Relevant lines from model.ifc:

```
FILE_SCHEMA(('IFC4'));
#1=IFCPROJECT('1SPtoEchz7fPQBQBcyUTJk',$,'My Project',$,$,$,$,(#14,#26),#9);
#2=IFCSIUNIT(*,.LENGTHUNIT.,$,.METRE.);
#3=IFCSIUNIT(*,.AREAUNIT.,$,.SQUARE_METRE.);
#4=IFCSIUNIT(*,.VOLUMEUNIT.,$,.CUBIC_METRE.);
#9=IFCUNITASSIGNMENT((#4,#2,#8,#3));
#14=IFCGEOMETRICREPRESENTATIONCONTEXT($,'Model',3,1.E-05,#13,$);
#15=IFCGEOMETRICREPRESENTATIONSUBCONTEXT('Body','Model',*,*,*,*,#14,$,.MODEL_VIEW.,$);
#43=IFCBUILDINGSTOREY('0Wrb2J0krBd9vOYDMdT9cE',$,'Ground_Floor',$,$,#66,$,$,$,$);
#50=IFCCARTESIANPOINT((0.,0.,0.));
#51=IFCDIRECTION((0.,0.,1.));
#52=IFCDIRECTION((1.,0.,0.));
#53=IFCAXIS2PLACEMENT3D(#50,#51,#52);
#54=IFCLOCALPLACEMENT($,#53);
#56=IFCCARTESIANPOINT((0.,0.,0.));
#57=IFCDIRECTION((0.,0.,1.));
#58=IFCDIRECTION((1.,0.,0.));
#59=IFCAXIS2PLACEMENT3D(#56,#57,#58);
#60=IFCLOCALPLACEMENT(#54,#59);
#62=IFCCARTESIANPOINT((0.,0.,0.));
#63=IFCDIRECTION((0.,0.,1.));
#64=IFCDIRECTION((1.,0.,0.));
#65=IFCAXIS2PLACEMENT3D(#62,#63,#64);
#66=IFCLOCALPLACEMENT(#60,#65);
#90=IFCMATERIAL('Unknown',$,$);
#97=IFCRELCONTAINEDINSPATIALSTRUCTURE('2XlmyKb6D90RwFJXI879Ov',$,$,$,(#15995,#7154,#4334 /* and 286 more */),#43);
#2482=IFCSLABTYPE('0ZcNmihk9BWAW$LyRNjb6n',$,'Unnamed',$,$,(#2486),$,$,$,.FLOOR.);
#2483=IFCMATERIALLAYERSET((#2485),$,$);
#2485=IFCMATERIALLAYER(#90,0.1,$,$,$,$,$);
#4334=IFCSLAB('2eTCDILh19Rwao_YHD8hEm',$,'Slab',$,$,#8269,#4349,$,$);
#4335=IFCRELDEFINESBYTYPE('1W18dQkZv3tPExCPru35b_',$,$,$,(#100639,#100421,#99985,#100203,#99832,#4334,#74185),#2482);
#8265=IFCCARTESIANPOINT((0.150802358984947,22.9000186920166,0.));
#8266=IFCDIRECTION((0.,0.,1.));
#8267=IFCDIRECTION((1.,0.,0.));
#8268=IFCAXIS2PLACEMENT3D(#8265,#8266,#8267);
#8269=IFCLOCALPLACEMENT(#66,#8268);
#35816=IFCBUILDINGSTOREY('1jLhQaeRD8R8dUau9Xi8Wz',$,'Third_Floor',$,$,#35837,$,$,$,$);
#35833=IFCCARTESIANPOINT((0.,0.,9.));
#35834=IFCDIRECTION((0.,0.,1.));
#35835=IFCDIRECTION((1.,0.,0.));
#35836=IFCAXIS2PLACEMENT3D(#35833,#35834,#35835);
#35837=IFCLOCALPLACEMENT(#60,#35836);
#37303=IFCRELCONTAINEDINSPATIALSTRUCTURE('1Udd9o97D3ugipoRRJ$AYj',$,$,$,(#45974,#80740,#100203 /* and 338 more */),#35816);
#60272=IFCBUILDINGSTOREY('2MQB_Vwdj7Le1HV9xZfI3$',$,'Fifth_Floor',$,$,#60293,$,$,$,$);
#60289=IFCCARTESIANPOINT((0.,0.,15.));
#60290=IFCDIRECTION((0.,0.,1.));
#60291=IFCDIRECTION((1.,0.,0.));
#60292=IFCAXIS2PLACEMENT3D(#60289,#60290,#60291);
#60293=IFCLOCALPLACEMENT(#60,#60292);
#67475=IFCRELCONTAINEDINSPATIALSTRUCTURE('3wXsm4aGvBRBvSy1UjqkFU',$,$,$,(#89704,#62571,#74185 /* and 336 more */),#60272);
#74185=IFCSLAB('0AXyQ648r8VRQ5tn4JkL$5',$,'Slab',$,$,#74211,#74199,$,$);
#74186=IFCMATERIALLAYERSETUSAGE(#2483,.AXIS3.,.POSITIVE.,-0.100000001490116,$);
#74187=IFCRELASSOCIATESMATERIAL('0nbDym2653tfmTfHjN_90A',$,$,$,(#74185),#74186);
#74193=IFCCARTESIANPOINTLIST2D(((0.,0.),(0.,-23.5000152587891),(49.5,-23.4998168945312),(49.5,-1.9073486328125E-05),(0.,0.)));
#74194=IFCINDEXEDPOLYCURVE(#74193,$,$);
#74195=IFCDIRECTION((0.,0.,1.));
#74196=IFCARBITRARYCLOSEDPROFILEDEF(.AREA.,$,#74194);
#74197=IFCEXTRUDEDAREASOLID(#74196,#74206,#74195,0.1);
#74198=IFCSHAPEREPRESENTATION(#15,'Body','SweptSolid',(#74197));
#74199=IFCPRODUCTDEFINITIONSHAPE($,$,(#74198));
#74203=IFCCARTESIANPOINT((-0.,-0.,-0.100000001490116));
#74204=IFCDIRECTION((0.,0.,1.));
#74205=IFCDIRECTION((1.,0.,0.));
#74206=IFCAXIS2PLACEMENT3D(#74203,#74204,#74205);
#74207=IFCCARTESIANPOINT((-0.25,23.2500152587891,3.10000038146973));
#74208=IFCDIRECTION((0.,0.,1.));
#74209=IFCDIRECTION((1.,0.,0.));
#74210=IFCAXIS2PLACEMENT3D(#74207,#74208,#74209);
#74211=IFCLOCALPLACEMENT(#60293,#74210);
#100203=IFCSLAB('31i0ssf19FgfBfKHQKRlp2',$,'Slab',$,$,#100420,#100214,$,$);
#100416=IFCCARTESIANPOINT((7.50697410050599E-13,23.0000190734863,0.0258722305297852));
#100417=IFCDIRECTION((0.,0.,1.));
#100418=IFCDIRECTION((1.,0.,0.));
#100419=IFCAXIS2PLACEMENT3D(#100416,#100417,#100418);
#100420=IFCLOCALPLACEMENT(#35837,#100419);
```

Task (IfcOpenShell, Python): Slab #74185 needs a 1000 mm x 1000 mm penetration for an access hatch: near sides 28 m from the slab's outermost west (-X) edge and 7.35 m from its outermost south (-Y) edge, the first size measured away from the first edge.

```python
import numpy as np
import ifcopenshell
import ifcopenshell.api.feature
import ifcopenshell.api.geometry
import ifcopenshell.api.root
import ifcopenshell.geom
import ifcopenshell.util.placement
import ifcopenshell.util.representation
import ifcopenshell.util.shape
import ifcopenshell.util.unit

model = ifcopenshell.open("model.ifc")
unit_scale = ifcopenshell.util.unit.calculate_unit_scale(model)
settings = ifcopenshell.geom.settings()


def volume(element):
    """Net volume in cubic metres, openings subtracted."""
    shape = ifcopenshell.geom.create_shape(settings, element)
    return ifcopenshell.util.shape.get_volume(shape.geometry)


slab = model.by_guid("0AXyQ648r8VRQ5tn4JkL$5")
before = volume(slab)

# Extent in the slab's own axes, in metres. The edges named are its -X and -Y sides.
slab_shape = ifcopenshell.geom.create_shape(settings, slab)
vertices = ifcopenshell.util.shape.get_vertices(slab_shape.geometry)
x_min, y_min, bottom = vertices.min(axis=0)
top = vertices[:, 2].max()

opening = ifcopenshell.api.root.create_entity(model, ifc_class="IfcOpeningElement", name="Access hatch opening", predefined_type="OPENING")
context = ifcopenshell.util.representation.get_context(model, "Model", "Body", "MODEL_VIEW")
width, depth = 1, 1
outline = [(0.0, 0.0), (width, 0.0), (width, depth), (0.0, depth), (0.0, 0.0)]
# Overshoot both faces by 50 mm so the cut is clean.
shape = ifcopenshell.api.geometry.add_slab_representation(
    model, context=context, depth=top - bottom + 0.1, polyline=outline
)
ifcopenshell.api.geometry.assign_representation(model, product=opening, representation=shape)

matrix = ifcopenshell.util.placement.get_local_placement(slab.ObjectPlacement)
matrix[:, 3] = matrix @ np.append(np.array([x_min + 28, y_min + 7.35, bottom - 0.05]) / unit_scale, 1.0)
ifcopenshell.api.geometry.edit_object_placement(model, product=opening, matrix=matrix, is_si=False)
ifcopenshell.api.feature.add_feature(model, feature=opening, element=slab)

after = volume(slab)

print(f"slab volume {before:.3f} -> {after:.3f} m3")

model.write("model_rev.ifc")
```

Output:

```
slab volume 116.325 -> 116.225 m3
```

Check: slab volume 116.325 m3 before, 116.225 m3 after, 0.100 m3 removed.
